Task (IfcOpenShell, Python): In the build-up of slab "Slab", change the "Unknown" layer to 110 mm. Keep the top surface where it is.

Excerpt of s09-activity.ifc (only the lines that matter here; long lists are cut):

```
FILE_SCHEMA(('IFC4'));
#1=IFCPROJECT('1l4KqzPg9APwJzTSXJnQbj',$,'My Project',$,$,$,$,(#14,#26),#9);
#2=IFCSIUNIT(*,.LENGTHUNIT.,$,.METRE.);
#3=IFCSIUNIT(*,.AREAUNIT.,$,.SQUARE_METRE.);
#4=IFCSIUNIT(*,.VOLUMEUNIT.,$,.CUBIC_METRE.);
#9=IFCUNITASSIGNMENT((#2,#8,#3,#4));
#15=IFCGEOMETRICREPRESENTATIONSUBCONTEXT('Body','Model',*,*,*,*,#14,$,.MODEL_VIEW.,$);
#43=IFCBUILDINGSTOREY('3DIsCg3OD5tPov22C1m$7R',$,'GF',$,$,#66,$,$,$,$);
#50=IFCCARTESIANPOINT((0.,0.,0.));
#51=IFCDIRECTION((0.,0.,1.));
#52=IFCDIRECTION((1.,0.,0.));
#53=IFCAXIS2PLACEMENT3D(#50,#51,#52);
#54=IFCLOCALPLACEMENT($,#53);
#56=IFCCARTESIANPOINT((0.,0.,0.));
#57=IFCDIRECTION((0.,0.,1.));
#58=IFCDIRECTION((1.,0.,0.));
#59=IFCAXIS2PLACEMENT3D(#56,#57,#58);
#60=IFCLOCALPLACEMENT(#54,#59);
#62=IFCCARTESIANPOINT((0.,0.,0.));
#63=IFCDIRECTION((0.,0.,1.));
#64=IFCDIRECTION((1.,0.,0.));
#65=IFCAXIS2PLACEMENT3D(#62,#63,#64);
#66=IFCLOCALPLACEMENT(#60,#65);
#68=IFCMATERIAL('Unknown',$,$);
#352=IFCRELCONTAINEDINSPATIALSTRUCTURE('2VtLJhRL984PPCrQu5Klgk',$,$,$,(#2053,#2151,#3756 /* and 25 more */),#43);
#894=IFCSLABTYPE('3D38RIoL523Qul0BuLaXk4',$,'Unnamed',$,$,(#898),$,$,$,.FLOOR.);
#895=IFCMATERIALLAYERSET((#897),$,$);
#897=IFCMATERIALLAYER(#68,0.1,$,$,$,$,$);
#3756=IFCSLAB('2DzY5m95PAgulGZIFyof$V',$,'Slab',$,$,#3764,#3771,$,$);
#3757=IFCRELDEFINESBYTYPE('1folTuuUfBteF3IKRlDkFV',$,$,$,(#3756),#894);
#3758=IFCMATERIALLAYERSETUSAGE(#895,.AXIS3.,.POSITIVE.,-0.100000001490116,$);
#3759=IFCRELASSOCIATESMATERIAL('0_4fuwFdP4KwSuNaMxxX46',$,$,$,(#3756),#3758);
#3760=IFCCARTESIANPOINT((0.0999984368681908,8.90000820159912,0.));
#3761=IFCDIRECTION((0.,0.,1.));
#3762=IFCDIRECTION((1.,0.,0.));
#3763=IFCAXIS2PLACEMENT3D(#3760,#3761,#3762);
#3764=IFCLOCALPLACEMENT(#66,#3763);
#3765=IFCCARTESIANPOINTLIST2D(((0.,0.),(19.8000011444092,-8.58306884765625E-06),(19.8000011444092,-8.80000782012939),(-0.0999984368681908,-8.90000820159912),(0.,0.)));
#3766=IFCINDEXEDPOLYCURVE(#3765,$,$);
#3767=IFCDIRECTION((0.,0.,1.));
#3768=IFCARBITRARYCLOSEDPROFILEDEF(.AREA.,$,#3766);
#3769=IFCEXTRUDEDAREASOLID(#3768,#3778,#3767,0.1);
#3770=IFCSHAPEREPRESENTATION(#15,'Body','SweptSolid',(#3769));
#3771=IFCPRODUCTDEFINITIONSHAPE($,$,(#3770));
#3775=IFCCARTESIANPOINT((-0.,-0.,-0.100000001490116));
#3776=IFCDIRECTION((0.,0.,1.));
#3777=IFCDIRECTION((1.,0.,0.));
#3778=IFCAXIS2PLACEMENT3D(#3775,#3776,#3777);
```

```python
import ifcopenshell
import ifcopenshell.util.element
import ifcopenshell.util.representation

model = ifcopenshell.open("s09-activity.ifc")

layer_set = model.by_id(895)
layer = next(l for l in layer_set.MaterialLayers if l.Material and l.Material.Name == "Unknown")
change = 0.11 - layer.LayerThickness
layer.LayerThickness += change

# Geometry does not follow the layer set by itself.
slabs = [e for e in ifcopenshell.util.element.get_elements_by_material(model, layer_set) if e.is_a("IfcSlab")]
for slab in sorted(slabs, key=lambda e: e.id()):
    body = ifcopenshell.util.representation.get_representation(slab, "Model", "Body")
    solid = body.Items[0]
    old_depth = solid.Depth
    solid.Depth += change
    # Extruded upwards: lower the start of the extrusion so the top stays.
    x, y, z = solid.Position.Location.Coordinates
    solid.Position.Location = model.createIfcCartesianPoint((x, y, z - change))
    print(slab.id(), f"{old_depth:g} -> {solid.Depth:g}")

# The layers are counted up from the underside, which has moved.
for usage in {ifcopenshell.util.element.get_material(slab) for slab in slabs}:
    usage.OffsetFromReferenceLine -= change

model.write("s09-activity-out.ifc")
```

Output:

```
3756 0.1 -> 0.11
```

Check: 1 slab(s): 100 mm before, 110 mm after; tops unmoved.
